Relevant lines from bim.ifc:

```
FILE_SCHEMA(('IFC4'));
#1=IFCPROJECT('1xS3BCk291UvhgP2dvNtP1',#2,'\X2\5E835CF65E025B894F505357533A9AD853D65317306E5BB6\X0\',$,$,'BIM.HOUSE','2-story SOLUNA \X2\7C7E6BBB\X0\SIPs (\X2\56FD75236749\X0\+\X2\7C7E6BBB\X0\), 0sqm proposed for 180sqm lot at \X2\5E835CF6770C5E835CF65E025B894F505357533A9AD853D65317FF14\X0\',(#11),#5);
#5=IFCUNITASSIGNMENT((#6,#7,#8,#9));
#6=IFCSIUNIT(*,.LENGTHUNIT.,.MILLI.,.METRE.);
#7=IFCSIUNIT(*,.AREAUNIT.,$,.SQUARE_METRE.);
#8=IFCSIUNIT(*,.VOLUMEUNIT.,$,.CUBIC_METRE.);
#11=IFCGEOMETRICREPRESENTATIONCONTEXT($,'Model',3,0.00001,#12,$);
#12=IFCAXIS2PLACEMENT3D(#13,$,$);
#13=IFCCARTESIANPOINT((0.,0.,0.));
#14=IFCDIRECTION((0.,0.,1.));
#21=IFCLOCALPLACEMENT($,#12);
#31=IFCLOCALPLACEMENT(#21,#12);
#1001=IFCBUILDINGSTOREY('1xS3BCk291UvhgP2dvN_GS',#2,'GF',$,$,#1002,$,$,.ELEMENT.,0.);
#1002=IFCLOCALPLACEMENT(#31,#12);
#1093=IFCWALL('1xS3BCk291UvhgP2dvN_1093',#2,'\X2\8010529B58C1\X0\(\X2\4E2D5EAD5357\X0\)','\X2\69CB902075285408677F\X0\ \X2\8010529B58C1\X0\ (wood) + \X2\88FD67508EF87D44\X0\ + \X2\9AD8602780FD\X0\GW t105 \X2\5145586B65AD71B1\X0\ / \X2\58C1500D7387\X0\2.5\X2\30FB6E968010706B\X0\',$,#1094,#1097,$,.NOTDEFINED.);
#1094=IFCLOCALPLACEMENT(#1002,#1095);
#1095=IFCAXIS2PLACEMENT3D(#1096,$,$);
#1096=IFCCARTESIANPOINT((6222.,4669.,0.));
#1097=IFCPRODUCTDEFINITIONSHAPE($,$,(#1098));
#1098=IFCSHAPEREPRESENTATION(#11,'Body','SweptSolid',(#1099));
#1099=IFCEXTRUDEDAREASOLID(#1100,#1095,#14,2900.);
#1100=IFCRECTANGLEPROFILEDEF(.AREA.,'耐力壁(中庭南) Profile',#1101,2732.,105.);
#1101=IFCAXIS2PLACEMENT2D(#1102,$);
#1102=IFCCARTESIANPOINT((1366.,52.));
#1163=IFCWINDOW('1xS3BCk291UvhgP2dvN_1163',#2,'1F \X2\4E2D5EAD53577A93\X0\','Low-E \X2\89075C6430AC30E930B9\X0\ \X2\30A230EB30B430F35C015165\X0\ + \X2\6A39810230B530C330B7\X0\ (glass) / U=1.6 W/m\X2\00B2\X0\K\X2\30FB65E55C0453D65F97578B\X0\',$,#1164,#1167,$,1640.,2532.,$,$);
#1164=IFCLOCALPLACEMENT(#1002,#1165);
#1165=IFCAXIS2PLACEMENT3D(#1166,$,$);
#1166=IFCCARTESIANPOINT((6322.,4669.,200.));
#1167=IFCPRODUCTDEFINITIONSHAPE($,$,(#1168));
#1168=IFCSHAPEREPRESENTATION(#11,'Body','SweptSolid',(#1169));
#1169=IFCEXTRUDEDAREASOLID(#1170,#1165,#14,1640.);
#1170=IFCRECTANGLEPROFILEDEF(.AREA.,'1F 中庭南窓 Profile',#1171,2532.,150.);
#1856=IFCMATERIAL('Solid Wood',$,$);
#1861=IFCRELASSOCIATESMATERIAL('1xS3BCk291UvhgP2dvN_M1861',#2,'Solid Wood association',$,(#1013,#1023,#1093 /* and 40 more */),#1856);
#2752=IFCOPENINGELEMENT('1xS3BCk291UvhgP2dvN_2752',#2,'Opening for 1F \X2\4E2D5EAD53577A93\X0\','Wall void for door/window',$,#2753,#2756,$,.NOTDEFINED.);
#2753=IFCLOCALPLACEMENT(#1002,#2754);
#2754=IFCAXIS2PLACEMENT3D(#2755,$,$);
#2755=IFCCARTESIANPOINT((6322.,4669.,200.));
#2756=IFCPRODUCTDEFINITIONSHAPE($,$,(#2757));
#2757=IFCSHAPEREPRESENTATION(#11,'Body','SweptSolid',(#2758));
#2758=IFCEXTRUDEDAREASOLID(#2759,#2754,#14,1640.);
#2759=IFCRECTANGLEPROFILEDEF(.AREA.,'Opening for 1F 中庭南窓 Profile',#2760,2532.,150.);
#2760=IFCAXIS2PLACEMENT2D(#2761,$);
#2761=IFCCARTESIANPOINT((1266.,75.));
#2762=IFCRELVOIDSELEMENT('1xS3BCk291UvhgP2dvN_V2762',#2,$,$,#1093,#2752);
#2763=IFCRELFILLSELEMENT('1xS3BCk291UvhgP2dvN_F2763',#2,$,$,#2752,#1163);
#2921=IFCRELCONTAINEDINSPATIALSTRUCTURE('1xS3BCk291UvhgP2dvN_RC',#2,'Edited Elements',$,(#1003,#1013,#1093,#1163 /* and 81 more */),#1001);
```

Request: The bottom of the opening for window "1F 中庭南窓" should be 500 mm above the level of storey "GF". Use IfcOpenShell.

```python
import numpy as np
import ifcopenshell
import ifcopenshell.api.geometry
import ifcopenshell.geom
import ifcopenshell.util.element
import ifcopenshell.util.placement
import ifcopenshell.util.shape
import ifcopenshell.util.unit

model = ifcopenshell.open("bim.ifc")
unit_scale = ifcopenshell.util.unit.calculate_unit_scale(model)

window = model.by_id(1163)
opening = window.FillsVoids[0].RelatingOpeningElement
storey = ifcopenshell.util.element.get_container(window, ifc_class="IfcBuildingStorey")
level = ifcopenshell.util.placement.get_local_placement(storey.ObjectPlacement)[2, 3]

# The opening's origin need not be at the sill, so measure its lowest point.
shape = ifcopenshell.geom.create_shape(ifcopenshell.geom.settings(), opening)
bottom = ifcopenshell.util.shape.get_shape_bottom_elevation(shape, shape.geometry) / unit_scale
dz = level + 0.5 / unit_scale - bottom

shift = np.array([0.0, 0.0, dz])
# The window is not placed relative to its opening, so move both.
for product in (opening, window):
    matrix = ifcopenshell.util.placement.get_local_placement(product.ObjectPlacement)
    matrix[:3, 3] += shift
    ifcopenshell.api.geometry.edit_object_placement(model, product=product, matrix=matrix, is_si=False)

print(f"moved by {dz * unit_scale:+.3f} m")

model.write("bim_rev.ifc")
```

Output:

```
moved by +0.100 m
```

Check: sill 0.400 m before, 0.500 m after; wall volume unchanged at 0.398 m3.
